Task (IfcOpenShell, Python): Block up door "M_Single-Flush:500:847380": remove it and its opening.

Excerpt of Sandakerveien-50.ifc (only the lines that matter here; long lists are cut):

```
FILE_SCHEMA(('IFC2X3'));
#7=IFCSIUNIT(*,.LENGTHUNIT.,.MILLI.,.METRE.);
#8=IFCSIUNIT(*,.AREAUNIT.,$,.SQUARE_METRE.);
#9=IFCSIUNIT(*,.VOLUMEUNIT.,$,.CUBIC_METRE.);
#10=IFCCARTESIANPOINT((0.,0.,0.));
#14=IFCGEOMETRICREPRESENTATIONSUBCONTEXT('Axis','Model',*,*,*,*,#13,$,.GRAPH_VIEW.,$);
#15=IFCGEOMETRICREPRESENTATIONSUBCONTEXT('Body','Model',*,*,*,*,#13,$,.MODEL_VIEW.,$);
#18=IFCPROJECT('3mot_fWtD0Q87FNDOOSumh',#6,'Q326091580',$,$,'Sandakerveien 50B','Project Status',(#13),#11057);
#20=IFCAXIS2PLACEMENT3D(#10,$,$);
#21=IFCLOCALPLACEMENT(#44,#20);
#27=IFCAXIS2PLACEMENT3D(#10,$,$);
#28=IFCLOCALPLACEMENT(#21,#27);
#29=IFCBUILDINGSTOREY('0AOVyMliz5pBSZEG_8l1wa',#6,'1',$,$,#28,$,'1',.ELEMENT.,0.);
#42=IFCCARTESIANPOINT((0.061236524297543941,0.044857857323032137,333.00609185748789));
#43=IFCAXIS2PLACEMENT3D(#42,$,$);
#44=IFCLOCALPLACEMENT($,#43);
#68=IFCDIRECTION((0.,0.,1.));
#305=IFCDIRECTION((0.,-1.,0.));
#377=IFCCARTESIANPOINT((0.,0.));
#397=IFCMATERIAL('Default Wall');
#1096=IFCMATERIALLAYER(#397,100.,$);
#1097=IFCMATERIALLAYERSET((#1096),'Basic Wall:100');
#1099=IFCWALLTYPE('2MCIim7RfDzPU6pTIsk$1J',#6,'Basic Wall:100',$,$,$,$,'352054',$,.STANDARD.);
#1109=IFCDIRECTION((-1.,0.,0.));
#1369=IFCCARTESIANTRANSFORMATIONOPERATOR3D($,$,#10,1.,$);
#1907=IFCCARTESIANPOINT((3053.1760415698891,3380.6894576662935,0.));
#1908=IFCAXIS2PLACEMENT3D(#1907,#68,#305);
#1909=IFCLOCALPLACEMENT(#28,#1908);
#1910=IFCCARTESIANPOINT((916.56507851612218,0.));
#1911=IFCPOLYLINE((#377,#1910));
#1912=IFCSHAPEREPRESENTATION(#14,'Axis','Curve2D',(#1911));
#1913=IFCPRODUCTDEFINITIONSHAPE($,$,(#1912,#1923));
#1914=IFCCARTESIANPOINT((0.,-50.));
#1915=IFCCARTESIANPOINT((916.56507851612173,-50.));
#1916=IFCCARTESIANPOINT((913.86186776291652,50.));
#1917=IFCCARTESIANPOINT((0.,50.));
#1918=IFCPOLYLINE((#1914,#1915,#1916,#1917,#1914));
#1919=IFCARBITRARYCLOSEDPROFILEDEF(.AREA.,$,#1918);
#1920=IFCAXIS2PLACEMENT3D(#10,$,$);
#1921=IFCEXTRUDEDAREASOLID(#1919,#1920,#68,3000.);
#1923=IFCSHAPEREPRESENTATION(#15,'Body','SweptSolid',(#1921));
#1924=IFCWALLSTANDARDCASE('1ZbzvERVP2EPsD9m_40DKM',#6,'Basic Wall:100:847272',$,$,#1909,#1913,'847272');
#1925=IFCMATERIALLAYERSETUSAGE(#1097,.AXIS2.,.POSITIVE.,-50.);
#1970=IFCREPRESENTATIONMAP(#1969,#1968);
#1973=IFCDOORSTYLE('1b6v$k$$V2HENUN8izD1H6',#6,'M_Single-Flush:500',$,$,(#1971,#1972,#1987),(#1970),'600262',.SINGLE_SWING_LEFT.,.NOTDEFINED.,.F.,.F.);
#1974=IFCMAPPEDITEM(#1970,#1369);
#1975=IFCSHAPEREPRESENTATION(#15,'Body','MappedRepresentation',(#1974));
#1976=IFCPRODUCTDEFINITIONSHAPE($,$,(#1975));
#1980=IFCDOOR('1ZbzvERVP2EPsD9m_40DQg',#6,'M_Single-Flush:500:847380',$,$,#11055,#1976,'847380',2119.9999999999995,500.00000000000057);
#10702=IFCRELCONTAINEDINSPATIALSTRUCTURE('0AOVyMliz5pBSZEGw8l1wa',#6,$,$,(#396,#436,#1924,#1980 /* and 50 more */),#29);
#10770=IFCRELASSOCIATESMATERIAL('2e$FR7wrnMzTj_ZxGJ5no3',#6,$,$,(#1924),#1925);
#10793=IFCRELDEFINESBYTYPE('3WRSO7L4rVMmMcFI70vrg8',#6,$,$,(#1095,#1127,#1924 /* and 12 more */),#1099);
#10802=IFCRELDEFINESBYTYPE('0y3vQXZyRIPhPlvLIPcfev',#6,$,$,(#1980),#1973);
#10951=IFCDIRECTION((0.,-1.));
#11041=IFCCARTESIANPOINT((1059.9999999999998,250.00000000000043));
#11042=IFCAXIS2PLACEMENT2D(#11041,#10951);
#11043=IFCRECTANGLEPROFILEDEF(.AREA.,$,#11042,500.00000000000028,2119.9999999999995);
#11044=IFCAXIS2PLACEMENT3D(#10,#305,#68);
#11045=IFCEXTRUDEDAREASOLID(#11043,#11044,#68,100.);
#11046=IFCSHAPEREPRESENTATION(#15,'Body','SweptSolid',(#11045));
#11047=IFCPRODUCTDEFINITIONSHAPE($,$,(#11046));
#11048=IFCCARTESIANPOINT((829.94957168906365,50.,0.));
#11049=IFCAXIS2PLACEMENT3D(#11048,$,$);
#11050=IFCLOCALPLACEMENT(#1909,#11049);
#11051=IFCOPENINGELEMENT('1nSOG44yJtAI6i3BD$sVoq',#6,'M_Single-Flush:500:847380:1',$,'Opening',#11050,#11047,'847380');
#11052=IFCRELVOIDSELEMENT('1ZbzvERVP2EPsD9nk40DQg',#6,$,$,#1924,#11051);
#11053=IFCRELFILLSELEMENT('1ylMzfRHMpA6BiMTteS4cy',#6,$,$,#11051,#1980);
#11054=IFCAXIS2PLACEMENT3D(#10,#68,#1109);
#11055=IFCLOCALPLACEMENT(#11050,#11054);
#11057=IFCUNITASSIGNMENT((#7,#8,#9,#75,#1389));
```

```python
import ifcopenshell
import ifcopenshell.api.feature
import ifcopenshell.api.root
import ifcopenshell.geom
import ifcopenshell.util.shape

model = ifcopenshell.open("Sandakerveien-50.ifc")
settings = ifcopenshell.geom.settings()


def volume(element):
    """Net volume in cubic metres, openings subtracted."""
    shape = ifcopenshell.geom.create_shape(settings, element)
    return ifcopenshell.util.shape.get_volume(shape.geometry)


door = model.by_guid("1ZbzvERVP2EPsD9m_40DQg")
opening = door.FillsVoids[0].RelatingOpeningElement
wall = opening.VoidsElements[0].RelatingBuildingElement
before = volume(wall)

ifcopenshell.api.root.remove_product(model, product=door)
ifcopenshell.api.feature.remove_feature(model, feature=opening)

after = volume(wall)

print(f"wall volume {before:.3f} -> {after:.3f} m3")

model.write("Sandakerveien-50_updated.ifc")
```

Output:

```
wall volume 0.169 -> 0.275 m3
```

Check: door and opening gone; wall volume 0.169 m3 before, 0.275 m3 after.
